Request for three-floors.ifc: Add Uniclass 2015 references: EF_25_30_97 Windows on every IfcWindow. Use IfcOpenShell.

First a look at what the model holds.

```python
import ifcopenshell

model = ifcopenshell.open("three-floors.ifc")
print(model.schema)
print("classifications:", [c.Name for c in model.by_type("IfcClassification")])
for ifc_class in ("IfcDoor", "IfcRoof", "IfcStair", "IfcWall", "IfcWindow"):
    print(ifc_class, len(model.by_type(ifc_class)))
```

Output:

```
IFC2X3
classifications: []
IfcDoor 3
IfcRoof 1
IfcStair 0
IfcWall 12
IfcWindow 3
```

```python
import ifcopenshell
import ifcopenshell.api.classification

model = ifcopenshell.open("three-floors.ifc")

# IFC2X3 requires Source and Edition and has no link from the project to the system.
system = model.create_entity("IfcClassification", Source="NBS", Edition="2015", Name="Uniclass 2015")

codes = {
    "IfcWindow": ("EF_25_30_97", "Windows"),
}
for ifc_class, (code, name) in codes.items():
    products = model.by_type(ifc_class)
    ifcopenshell.api.classification.add_reference(
        model, products=products, classification=system, identification=code, name=name
    )
    print(code, len(products))

model.write("three-floors_edited.ifc")
```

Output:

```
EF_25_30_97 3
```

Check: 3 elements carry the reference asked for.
